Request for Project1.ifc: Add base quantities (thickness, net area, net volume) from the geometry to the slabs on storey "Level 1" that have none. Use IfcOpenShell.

First a look at what the model holds.

```python
import ifcopenshell
import ifcopenshell.util.element
import ifcopenshell.util.unit

model = ifcopenshell.open("Project1.ifc")
print(model.schema)
for unit_type in ("LENGTHUNIT", "AREAUNIT", "VOLUMEUNIT"):
    print(unit_type, ifcopenshell.util.unit.calculate_unit_scale(model, unit_type))
storey = next(s for s in model.by_type("IfcBuildingStorey") if s.Name == "Level 1")
slabs = [e for e in ifcopenshell.util.element.get_decomposition(storey) if e.is_a("IfcSlab")]
for e in sorted(slabs, key=lambda e: e.id()):
    print(e.id(), e.is_a(), e.Name, list(ifcopenshell.util.element.get_psets(e, qtos_only=True)), sep=" | ")
```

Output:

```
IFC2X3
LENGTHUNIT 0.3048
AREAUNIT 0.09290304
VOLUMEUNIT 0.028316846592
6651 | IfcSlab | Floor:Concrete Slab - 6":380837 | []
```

```python
import ifcopenshell
import ifcopenshell.api.pset
import ifcopenshell.geom
import ifcopenshell.util.element
import ifcopenshell.util.shape
import ifcopenshell.util.unit

model = ifcopenshell.open("Project1.ifc")
unit_scale = ifcopenshell.util.unit.calculate_unit_scale(model)
area_scale = ifcopenshell.util.unit.calculate_unit_scale(model, "AREAUNIT")
volume_scale = ifcopenshell.util.unit.calculate_unit_scale(model, "VOLUMEUNIT")
settings = ifcopenshell.geom.settings()

storey = next(s for s in model.by_type("IfcBuildingStorey") if s.Name == "Level 1")
slabs = [e for e in ifcopenshell.util.element.get_decomposition(storey) if e.is_a("IfcSlab")]

for e in sorted(slabs, key=lambda e: e.id()):
    if ifcopenshell.util.element.get_psets(e, qtos_only=True, should_inherit=False):
        continue
    # Geometry comes back in metres, in the element's own axes.
    shape = ifcopenshell.geom.create_shape(settings, e)
    values = {
        "Width": ifcopenshell.util.shape.get_z(shape.geometry) / unit_scale,
        "NetArea": ifcopenshell.util.shape.get_footprint_area(shape.geometry) / area_scale,
        "NetVolume": ifcopenshell.util.shape.get_volume(shape.geometry) / volume_scale,
    }
    qto = ifcopenshell.api.pset.add_qto(model, product=e, name="BaseQuantities")
    ifcopenshell.api.pset.edit_qto(model, qto=qto, properties=values)
    print(e.id(), {k: round(v, 3) for k, v in values.items()})

model.write("Project1-out.ifc")
```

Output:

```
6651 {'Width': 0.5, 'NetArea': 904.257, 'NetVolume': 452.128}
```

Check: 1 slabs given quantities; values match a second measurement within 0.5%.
